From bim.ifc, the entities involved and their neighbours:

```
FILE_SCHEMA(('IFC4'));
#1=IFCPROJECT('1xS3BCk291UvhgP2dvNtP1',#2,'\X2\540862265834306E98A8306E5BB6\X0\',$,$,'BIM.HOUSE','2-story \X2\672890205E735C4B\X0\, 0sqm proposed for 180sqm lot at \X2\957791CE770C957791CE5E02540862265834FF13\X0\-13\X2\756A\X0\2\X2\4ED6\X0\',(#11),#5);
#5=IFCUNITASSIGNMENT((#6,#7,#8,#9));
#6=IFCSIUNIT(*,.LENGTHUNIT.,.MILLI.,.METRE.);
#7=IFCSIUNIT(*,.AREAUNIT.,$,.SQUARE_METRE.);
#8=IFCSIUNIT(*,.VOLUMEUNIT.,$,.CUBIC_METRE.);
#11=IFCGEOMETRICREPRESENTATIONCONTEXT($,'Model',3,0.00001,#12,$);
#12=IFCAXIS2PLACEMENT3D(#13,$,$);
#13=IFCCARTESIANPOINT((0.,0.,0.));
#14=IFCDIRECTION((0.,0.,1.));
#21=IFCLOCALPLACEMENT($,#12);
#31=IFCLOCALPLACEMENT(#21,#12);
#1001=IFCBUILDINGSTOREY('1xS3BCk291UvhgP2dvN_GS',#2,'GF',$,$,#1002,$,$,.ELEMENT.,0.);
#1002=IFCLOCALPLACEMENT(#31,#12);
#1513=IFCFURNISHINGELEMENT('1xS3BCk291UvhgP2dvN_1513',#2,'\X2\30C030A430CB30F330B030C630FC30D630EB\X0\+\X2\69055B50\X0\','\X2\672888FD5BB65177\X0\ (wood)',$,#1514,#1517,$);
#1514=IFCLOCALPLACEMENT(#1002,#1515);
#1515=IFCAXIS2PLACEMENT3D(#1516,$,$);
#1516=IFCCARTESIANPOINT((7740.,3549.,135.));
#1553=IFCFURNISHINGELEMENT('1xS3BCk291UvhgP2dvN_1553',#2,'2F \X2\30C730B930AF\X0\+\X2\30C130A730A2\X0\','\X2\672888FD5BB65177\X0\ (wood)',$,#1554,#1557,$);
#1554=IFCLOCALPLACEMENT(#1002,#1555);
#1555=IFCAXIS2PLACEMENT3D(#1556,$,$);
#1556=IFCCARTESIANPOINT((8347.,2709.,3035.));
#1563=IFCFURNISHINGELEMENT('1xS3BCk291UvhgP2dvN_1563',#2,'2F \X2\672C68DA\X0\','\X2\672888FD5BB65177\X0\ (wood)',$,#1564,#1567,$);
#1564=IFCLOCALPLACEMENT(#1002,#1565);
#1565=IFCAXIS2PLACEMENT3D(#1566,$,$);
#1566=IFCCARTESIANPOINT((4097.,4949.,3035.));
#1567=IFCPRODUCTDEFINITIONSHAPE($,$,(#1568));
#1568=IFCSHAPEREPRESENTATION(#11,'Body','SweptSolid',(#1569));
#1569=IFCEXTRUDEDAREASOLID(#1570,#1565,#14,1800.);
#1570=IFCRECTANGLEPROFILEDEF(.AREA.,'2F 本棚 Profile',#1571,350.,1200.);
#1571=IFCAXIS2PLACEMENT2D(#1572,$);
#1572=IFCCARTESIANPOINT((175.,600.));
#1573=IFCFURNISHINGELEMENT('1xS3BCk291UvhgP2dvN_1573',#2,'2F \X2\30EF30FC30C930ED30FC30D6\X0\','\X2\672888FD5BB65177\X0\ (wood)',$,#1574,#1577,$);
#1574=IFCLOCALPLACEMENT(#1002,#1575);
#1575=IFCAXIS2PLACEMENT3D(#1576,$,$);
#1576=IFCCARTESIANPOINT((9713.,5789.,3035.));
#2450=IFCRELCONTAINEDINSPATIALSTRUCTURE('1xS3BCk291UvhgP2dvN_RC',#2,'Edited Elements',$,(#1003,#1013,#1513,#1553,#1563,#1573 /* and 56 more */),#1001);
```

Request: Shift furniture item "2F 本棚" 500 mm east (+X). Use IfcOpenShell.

```python
import ifcopenshell
import ifcopenshell.api.geometry
import ifcopenshell.util.placement
import ifcopenshell.util.unit

model = ifcopenshell.open("bim.ifc")
unit_scale = ifcopenshell.util.unit.calculate_unit_scale(model)

item = model.by_guid("1xS3BCk291UvhgP2dvN_1563")
matrix = ifcopenshell.util.placement.get_local_placement(item.ObjectPlacement)
matrix[0, 3] += 0.5 / unit_scale
ifcopenshell.api.geometry.edit_object_placement(model, product=item, matrix=matrix, is_si=False)

print(ifcopenshell.util.placement.get_local_placement(item.ObjectPlacement).round(3) + 0.0)

model.write("bim_rev.ifc")
```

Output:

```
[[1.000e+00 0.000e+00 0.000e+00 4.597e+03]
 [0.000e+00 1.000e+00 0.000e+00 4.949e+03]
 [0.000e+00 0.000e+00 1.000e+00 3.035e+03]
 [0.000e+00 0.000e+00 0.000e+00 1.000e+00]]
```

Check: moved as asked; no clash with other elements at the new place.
